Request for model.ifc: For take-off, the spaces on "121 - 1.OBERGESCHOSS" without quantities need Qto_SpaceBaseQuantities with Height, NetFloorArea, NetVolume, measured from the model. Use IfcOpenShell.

First a look at what the model holds.

```python
import ifcopenshell
import ifcopenshell.util.element
import ifcopenshell.util.unit

model = ifcopenshell.open("model.ifc")
print(model.schema)
for unit_type in ("LENGTHUNIT", "AREAUNIT", "VOLUMEUNIT"):
    print(unit_type, ifcopenshell.util.unit.calculate_unit_scale(model, unit_type))
storey = next(s for s in model.by_type("IfcBuildingStorey") if s.Name == "121 - 1.OBERGESCHOSS")
spaces = [e for e in ifcopenshell.util.element.get_decomposition(storey) if e.is_a("IfcSpace")]
for e in sorted(spaces, key=lambda e: e.id()):
    print(e.id(), e.is_a(), e.Name, list(ifcopenshell.util.element.get_psets(e, qtos_only=True)), sep=" | ")
```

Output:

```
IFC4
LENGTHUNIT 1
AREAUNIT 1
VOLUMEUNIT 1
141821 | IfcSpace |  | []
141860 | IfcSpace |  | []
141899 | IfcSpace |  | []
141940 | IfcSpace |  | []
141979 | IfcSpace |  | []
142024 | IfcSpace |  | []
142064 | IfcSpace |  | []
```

```python
import ifcopenshell
import ifcopenshell.api.pset
import ifcopenshell.geom
import ifcopenshell.util.element
import ifcopenshell.util.shape
import ifcopenshell.util.unit

model = ifcopenshell.open("model.ifc")
unit_scale = ifcopenshell.util.unit.calculate_unit_scale(model)
area_scale = ifcopenshell.util.unit.calculate_unit_scale(model, "AREAUNIT")
volume_scale = ifcopenshell.util.unit.calculate_unit_scale(model, "VOLUMEUNIT")
settings = ifcopenshell.geom.settings()

storey = next(s for s in model.by_type("IfcBuildingStorey") if s.Name == "121 - 1.OBERGESCHOSS")
spaces = [e for e in ifcopenshell.util.element.get_decomposition(storey) if e.is_a("IfcSpace")]

for e in sorted(spaces, key=lambda e: e.id()):
    if ifcopenshell.util.element.get_psets(e, qtos_only=True, should_inherit=False):
        continue
    # Geometry comes back in metres, in the element's own axes.
    shape = ifcopenshell.geom.create_shape(settings, e)
    values = {
        "Height": ifcopenshell.util.shape.get_z(shape.geometry) / unit_scale,
        "NetFloorArea": ifcopenshell.util.shape.get_footprint_area(shape.geometry) / area_scale,
        "NetVolume": ifcopenshell.util.shape.get_volume(shape.geometry) / volume_scale,
    }
    qto = ifcopenshell.api.pset.add_qto(model, product=e, name="Qto_SpaceBaseQuantities")
    ifcopenshell.api.pset.edit_qto(model, qto=qto, properties=values)
    print(e.id(), {k: round(v, 3) for k, v in values.items()})

model.write("model_updated.ifc")
```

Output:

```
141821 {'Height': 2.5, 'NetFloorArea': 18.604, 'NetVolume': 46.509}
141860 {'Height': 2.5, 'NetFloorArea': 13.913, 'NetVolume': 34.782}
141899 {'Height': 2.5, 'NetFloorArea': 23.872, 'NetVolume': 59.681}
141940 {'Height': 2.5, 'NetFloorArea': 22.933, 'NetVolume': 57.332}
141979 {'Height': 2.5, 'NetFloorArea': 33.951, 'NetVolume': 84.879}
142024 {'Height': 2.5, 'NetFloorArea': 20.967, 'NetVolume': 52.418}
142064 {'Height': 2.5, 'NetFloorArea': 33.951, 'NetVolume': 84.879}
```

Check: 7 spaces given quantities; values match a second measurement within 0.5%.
